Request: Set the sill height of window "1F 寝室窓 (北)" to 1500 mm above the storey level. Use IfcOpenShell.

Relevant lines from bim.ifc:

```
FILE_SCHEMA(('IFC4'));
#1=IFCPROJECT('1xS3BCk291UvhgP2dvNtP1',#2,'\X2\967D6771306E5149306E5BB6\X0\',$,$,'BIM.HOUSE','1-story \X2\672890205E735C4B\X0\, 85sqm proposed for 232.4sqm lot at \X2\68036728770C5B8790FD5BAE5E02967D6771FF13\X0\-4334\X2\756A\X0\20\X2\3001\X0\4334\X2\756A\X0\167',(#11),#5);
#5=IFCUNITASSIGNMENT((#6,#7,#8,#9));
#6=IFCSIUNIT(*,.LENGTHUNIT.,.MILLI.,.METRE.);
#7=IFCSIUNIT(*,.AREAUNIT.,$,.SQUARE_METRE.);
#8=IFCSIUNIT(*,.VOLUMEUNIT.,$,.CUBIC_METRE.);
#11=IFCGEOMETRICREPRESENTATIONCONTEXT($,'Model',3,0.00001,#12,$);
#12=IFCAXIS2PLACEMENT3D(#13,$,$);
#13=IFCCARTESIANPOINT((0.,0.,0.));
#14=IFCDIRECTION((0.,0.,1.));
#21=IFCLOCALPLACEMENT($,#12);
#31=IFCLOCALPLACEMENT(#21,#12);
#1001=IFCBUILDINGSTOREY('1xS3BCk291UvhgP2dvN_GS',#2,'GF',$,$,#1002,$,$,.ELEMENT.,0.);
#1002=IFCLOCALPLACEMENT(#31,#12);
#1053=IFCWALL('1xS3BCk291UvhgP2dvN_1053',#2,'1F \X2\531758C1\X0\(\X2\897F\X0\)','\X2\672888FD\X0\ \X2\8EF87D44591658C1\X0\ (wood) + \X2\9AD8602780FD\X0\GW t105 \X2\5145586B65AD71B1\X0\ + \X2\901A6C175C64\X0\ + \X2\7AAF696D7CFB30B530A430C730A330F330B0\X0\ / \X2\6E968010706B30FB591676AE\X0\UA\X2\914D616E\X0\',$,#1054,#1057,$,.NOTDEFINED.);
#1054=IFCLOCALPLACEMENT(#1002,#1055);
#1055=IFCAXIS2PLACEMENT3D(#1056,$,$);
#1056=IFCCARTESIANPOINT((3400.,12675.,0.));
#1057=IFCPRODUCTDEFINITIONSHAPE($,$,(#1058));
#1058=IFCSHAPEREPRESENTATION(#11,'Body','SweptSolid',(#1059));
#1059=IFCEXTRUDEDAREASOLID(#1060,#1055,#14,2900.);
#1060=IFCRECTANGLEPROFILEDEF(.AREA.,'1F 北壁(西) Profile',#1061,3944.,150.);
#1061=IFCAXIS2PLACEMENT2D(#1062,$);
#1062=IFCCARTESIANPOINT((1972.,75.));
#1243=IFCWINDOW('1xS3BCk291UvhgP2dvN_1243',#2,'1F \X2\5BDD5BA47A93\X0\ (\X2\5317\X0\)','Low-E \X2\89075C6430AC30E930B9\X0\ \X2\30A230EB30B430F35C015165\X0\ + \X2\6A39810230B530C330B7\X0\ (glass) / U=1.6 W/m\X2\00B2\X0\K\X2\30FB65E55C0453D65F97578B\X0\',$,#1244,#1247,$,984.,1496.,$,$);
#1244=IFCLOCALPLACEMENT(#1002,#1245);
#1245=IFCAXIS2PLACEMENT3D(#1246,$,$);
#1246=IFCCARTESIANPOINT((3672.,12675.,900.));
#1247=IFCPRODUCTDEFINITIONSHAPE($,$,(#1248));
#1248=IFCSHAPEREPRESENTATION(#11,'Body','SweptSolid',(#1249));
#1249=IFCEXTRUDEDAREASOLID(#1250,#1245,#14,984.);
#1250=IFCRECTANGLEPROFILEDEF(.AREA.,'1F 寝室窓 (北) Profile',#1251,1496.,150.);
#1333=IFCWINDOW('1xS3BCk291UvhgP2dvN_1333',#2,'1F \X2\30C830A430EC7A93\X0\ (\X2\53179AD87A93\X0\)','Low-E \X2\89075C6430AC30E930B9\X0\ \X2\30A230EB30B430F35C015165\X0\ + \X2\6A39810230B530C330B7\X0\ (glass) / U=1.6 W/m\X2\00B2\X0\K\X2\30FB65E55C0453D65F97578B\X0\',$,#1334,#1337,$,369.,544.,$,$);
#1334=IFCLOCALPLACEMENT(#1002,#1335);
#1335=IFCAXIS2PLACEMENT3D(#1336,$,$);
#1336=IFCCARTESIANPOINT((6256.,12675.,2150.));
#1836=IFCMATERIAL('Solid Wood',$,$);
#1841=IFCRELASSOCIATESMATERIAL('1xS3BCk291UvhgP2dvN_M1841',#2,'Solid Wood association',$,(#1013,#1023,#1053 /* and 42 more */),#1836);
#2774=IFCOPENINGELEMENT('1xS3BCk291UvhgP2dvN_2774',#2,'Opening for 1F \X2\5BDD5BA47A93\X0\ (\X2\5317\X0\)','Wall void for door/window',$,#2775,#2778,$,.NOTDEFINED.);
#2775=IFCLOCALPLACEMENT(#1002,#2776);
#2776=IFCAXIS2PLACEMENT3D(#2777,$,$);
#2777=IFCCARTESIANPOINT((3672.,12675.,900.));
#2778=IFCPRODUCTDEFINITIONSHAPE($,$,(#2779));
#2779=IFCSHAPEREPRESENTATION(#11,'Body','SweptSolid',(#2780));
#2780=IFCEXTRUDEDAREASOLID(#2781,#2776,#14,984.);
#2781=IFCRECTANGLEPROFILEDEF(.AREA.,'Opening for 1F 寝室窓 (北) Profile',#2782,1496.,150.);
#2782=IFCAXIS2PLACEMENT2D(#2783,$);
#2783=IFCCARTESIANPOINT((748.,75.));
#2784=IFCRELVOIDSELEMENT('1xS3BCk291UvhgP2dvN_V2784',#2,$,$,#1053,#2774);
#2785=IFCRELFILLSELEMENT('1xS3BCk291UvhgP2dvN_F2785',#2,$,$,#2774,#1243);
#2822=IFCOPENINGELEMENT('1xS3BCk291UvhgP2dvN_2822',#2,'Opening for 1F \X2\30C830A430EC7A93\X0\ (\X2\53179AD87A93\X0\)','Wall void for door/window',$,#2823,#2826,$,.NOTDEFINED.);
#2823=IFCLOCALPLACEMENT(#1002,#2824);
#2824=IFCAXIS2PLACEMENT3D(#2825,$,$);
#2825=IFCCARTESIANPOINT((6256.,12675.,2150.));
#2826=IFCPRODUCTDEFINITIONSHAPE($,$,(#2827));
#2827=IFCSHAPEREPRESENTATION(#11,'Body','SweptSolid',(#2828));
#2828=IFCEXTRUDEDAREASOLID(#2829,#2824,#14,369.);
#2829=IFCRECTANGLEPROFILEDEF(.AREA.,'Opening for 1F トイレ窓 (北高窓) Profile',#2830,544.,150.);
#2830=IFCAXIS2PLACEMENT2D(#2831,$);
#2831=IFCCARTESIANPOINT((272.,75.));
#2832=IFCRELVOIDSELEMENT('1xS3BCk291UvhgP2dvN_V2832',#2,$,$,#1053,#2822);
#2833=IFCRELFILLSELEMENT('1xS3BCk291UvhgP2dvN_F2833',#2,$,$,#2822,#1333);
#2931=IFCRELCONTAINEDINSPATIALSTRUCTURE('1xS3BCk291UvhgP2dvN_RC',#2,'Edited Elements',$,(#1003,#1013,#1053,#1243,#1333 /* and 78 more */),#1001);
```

```python
import numpy as np
import ifcopenshell
import ifcopenshell.api.geometry
import ifcopenshell.geom
import ifcopenshell.util.element
import ifcopenshell.util.placement
import ifcopenshell.util.shape
import ifcopenshell.util.unit

model = ifcopenshell.open("bim.ifc")
unit_scale = ifcopenshell.util.unit.calculate_unit_scale(model)

window = model.by_guid("1xS3BCk291UvhgP2dvN_1243")
opening = window.FillsVoids[0].RelatingOpeningElement
storey = ifcopenshell.util.element.get_container(window, ifc_class="IfcBuildingStorey")
level = ifcopenshell.util.placement.get_local_placement(storey.ObjectPlacement)[2, 3]

# The opening's origin need not be at the sill, so measure its lowest point.
shape = ifcopenshell.geom.create_shape(ifcopenshell.geom.settings(), opening)
bottom = ifcopenshell.util.shape.get_shape_bottom_elevation(shape, shape.geometry) / unit_scale
dz = level + 1.5 / unit_scale - bottom

shift = np.array([0.0, 0.0, dz])
# The window is not placed relative to its opening, so move both.
for product in (opening, window):
    matrix = ifcopenshell.util.placement.get_local_placement(product.ObjectPlacement)
    matrix[:3, 3] += shift
    ifcopenshell.api.geometry.edit_object_placement(model, product=product, matrix=matrix, is_si=False)

print(f"moved by {dz * unit_scale:+.3f} m")

model.write("bim-out.ifc")
```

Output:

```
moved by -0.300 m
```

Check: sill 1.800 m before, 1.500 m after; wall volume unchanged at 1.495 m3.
